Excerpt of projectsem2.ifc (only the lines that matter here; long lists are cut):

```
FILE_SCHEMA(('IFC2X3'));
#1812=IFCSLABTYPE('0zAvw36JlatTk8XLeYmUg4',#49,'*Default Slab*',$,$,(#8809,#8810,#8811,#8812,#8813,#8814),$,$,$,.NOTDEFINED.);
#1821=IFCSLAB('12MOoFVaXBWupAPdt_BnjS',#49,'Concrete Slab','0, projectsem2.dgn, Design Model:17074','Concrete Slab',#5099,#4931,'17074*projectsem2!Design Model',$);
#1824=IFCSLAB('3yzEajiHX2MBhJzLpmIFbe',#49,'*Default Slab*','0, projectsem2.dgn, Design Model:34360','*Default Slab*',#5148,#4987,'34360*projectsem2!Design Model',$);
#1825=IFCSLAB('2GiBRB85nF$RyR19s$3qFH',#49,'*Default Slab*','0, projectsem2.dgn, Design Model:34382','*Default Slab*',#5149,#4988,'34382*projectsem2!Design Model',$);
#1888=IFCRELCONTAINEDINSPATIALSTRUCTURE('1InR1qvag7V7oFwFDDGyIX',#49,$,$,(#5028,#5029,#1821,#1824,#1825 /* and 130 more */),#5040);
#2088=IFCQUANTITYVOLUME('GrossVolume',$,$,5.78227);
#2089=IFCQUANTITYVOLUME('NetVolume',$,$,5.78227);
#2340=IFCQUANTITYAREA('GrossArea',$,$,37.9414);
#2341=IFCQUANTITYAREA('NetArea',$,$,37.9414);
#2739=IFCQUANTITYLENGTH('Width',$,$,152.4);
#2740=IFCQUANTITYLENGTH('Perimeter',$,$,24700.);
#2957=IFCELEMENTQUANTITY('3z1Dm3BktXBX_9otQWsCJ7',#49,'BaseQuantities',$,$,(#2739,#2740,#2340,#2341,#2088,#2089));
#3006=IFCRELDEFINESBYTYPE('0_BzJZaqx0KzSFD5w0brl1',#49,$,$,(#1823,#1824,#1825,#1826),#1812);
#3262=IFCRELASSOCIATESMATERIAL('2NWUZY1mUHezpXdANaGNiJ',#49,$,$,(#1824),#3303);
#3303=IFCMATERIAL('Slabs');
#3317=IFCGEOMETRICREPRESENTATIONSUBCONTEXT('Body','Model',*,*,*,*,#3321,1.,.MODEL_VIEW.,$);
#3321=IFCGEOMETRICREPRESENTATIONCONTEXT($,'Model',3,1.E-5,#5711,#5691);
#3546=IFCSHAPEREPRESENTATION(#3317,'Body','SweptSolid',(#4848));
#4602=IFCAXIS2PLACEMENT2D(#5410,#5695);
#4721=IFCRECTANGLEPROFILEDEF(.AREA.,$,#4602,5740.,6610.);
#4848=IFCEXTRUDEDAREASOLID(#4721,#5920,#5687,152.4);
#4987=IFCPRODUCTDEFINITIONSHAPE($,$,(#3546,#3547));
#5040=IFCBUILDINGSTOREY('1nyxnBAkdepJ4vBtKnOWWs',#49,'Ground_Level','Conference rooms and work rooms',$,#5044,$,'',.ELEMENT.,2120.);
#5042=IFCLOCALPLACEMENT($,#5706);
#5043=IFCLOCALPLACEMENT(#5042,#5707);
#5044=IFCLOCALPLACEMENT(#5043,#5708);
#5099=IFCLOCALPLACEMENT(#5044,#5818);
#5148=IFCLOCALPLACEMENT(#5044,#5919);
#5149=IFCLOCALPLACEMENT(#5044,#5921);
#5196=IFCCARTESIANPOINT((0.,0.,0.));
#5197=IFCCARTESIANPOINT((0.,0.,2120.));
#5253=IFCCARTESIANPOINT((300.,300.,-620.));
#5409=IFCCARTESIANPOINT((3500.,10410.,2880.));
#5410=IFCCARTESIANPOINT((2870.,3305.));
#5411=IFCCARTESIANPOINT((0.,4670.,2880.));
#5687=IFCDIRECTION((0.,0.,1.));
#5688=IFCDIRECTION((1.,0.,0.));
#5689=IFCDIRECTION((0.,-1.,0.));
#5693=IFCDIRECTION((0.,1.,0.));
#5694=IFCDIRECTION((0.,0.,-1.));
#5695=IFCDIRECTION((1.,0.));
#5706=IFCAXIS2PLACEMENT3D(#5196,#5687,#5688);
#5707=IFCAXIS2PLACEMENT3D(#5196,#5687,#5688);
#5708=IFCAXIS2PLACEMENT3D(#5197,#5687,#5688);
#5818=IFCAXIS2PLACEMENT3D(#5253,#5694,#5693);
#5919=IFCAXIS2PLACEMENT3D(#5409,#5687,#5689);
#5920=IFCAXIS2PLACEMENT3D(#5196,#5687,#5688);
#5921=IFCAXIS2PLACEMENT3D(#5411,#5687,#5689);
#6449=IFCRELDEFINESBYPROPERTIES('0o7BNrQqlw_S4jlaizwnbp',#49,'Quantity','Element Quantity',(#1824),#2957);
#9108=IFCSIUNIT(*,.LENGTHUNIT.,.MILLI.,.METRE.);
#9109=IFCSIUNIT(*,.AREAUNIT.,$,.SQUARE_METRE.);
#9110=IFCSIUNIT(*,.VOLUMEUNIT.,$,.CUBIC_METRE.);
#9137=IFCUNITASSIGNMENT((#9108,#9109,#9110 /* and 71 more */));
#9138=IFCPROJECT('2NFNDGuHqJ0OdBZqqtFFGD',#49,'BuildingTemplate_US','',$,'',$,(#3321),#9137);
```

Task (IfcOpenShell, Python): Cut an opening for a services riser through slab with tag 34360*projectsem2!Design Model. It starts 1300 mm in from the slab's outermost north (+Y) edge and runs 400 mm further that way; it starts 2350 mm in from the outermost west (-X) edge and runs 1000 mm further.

```python
import numpy as np
import ifcopenshell
import ifcopenshell.api.feature
import ifcopenshell.api.geometry
import ifcopenshell.api.pset
import ifcopenshell.api.root
import ifcopenshell.geom
import ifcopenshell.util.element
import ifcopenshell.util.placement
import ifcopenshell.util.representation
import ifcopenshell.util.shape
import ifcopenshell.util.unit

model = ifcopenshell.open("projectsem2.ifc")
unit_scale = ifcopenshell.util.unit.calculate_unit_scale(model)
area_scale = ifcopenshell.util.unit.calculate_unit_scale(model, "AREAUNIT")
volume_scale = ifcopenshell.util.unit.calculate_unit_scale(model, "VOLUMEUNIT")
settings = ifcopenshell.geom.settings()


def volume(element):
    """Net volume in cubic metres, openings subtracted."""
    shape = ifcopenshell.geom.create_shape(settings, element)
    return ifcopenshell.util.shape.get_volume(shape.geometry)


slab = model.by_guid("3yzEajiHX2MBhJzLpmIFbe")
before = volume(slab)

# Extent in the slab's own axes, in metres. The edges named are its -X and -Y sides.
slab_shape = ifcopenshell.geom.create_shape(settings, slab)
vertices = ifcopenshell.util.shape.get_vertices(slab_shape.geometry)
x_min, y_min, bottom = vertices.min(axis=0)
top = vertices[:, 2].max()

opening = ifcopenshell.api.root.create_entity(model, ifc_class="IfcOpeningElement", name="Services riser opening")
context = ifcopenshell.util.representation.get_context(model, "Model", "Body", "MODEL_VIEW")
width, depth = 0.4, 1
outline = [(0.0, 0.0), (width, 0.0), (width, depth), (0.0, depth), (0.0, 0.0)]
# Overshoot both faces by 50 mm so the cut is clean.
shape = ifcopenshell.api.geometry.add_slab_representation(
    model, context=context, depth=top - bottom + 0.1, polyline=outline
)
ifcopenshell.api.geometry.assign_representation(model, product=opening, representation=shape)

matrix = ifcopenshell.util.placement.get_local_placement(slab.ObjectPlacement)
matrix[:, 3] = matrix @ np.append(np.array([x_min + 1.3, y_min + 2.35, bottom - 0.05]) / unit_scale, 1.0)
ifcopenshell.api.geometry.edit_object_placement(model, product=opening, matrix=matrix, is_si=False)
ifcopenshell.api.feature.add_feature(model, feature=opening, element=slab)

after = volume(slab)

# Update the slab's stored quantities.
qto = model.by_id(ifcopenshell.util.element.get_pset(slab, "BaseQuantities", should_inherit=False)["id"])
ifcopenshell.api.pset.edit_qto(model, qto=qto, properties={
    "NetArea": after / (top - bottom) / area_scale,
    "NetVolume": after / volume_scale,
})

print(f"slab volume {before:.3f} -> {after:.3f} m3")

model.write("projectsem2_updated.ifc")
```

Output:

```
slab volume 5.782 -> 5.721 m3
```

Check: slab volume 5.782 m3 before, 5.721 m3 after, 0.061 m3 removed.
